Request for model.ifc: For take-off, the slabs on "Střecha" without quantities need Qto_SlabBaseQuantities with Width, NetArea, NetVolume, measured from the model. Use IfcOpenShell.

First a look at what the model holds.

```python
import ifcopenshell
import ifcopenshell.util.element
import ifcopenshell.util.unit

model = ifcopenshell.open("model.ifc")
print(model.schema)
for unit_type in ("LENGTHUNIT", "AREAUNIT", "VOLUMEUNIT"):
    print(unit_type, ifcopenshell.util.unit.calculate_unit_scale(model, unit_type))
storey = next(s for s in model.by_type("IfcBuildingStorey") if s.Name == "Střecha")
slabs = [e for e in ifcopenshell.util.element.get_decomposition(storey) if e.is_a("IfcSlab")]
for e in sorted(slabs, key=lambda e: e.id()):
    print(e.id(), e.is_a(), e.Name, list(ifcopenshell.util.element.get_psets(e, qtos_only=True)), sep=" | ")
```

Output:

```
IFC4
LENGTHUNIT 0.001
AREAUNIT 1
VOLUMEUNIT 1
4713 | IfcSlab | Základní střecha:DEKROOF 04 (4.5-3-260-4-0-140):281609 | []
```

```python
import ifcopenshell
import ifcopenshell.api.pset
import ifcopenshell.geom
import ifcopenshell.util.element
import ifcopenshell.util.shape
import ifcopenshell.util.unit

model = ifcopenshell.open("model.ifc")
unit_scale = ifcopenshell.util.unit.calculate_unit_scale(model)
area_scale = ifcopenshell.util.unit.calculate_unit_scale(model, "AREAUNIT")
volume_scale = ifcopenshell.util.unit.calculate_unit_scale(model, "VOLUMEUNIT")
settings = ifcopenshell.geom.settings()

storey = next(s for s in model.by_type("IfcBuildingStorey") if s.Name == "Střecha")
slabs = [e for e in ifcopenshell.util.element.get_decomposition(storey) if e.is_a("IfcSlab")]

for e in sorted(slabs, key=lambda e: e.id()):
    if ifcopenshell.util.element.get_psets(e, qtos_only=True, should_inherit=False):
        continue
    # Geometry comes back in metres, in the element's own axes.
    shape = ifcopenshell.geom.create_shape(settings, e)
    values = {
        "Width": ifcopenshell.util.shape.get_z(shape.geometry) / unit_scale,
        "NetArea": ifcopenshell.util.shape.get_footprint_area(shape.geometry) / area_scale,
        "NetVolume": ifcopenshell.util.shape.get_volume(shape.geometry) / volume_scale,
    }
    qto = ifcopenshell.api.pset.add_qto(model, product=e, name="Qto_SlabBaseQuantities")
    ifcopenshell.api.pset.edit_qto(model, qto=qto, properties=values)
    print(e.id(), {k: round(v, 3) for k, v in values.items()})

model.write("model-out.ifc")
```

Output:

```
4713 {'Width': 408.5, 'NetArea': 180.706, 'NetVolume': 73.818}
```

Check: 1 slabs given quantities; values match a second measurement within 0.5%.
